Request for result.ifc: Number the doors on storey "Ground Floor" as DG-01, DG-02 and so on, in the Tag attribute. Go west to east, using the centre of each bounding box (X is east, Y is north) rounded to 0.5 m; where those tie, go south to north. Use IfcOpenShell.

First a look at what the model holds.

```python
import ifcopenshell
import ifcopenshell.util.element
import ifcopenshell.util.placement

model = ifcopenshell.open("result.ifc")
print(model.schema)
storey = next(s for s in model.by_type("IfcBuildingStorey") if s.Name == "Ground Floor")
doors = [e for e in ifcopenshell.util.element.get_decomposition(storey) if e.is_a("IfcDoor")]
for e in sorted(doors, key=lambda e: e.id()):
    origin = ifcopenshell.util.placement.get_local_placement(e.ObjectPlacement)[:3, 3]
    print(e.id(), e.Tag, e.Name, origin.round(2) + 0.0, sep=" | ")
```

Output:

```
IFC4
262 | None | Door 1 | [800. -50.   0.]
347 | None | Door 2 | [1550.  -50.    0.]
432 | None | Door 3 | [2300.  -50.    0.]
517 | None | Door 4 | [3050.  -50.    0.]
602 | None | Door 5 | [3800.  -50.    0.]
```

```python
import ifcopenshell
import ifcopenshell.geom
import ifcopenshell.util.element
import ifcopenshell.util.shape

model = ifcopenshell.open("result.ifc")
settings = ifcopenshell.geom.settings()
settings.set("use-world-coords", True)


def centre(element):
    shape = ifcopenshell.geom.create_shape(settings, element)
    return ifcopenshell.util.shape.get_bbox_centroid(shape.geometry)


storey = next(s for s in model.by_type("IfcBuildingStorey") if s.Name == "Ground Floor")
doors = [e for e in ifcopenshell.util.element.get_decomposition(storey) if e.is_a("IfcDoor")]

# Insertion points can sit at a corner or the storey origin, so sort by the geometry (in metres).
centres = {e: centre(e) for e in doors}
doors.sort(key=lambda e: (round(centres[e][0] / 0.5), centres[e][1]))

for i, e in enumerate(doors, start=1):
    number = f"DG-{i:02d}"
    e.Tag = number
    print(e.id(), number)

model.write("result_edited.ifc")
```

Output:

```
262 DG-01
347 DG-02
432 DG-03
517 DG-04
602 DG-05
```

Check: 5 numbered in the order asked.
